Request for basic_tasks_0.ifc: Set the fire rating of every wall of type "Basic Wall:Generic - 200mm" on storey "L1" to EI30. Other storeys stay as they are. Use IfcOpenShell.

First a look at what the model holds.

```python
import ifcopenshell
import ifcopenshell.util.element

model = ifcopenshell.open("basic_tasks_0.ifc")
print(model.schema)
storey = next(s for s in model.by_type("IfcBuildingStorey") if s.Name == "L1")
walls = [e for e in ifcopenshell.util.element.get_decomposition(storey) if e.is_a("IfcWall")]
seen = {}
for e in walls:
    element_type = ifcopenshell.util.element.get_type(e)
    key = (element_type.Name if element_type != e and element_type else None, ifcopenshell.util.element.get_pset(e, "Pset_WallCommon", "FireRating"))
    seen[key] = seen.get(key, 0) + 1
for (name, value), count in sorted(seen.items(), key=str):
    print(count, "x", name, "|", value)
```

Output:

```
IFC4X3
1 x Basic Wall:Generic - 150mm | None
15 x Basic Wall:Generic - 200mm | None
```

```python
import ifcopenshell
import ifcopenshell.api.pset
import ifcopenshell.util.element

model = ifcopenshell.open("basic_tasks_0.ifc")

storey = next(s for s in model.by_type("IfcBuildingStorey") if s.Name == "L1")
walls = [e for e in ifcopenshell.util.element.get_decomposition(storey) if e.is_a("IfcWall")]

count = 0
for e in walls:
    element_type = ifcopenshell.util.element.get_type(e)
    if element_type in (None, e) or element_type.Name != "Basic Wall:Generic - 200mm":
        continue
    # add_pset returns the element's existing set when there is one.
    pset = ifcopenshell.api.pset.add_pset(model, product=e, name="Pset_WallCommon")
    ifcopenshell.api.pset.edit_pset(model, pset=pset, properties={"FireRating": "EI30"})
    count += 1

print(count, "walls updated")

model.write("basic_tasks_0_edited.ifc")
```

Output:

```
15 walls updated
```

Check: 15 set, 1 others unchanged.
